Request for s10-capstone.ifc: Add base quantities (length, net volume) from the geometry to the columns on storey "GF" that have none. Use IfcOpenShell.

First a look at what the model holds.

```python
import ifcopenshell
import ifcopenshell.util.element
import ifcopenshell.util.unit

model = ifcopenshell.open("s10-capstone.ifc")
print(model.schema)
for unit_type in ("LENGTHUNIT", "AREAUNIT", "VOLUMEUNIT"):
    print(unit_type, ifcopenshell.util.unit.calculate_unit_scale(model, unit_type))
storey = next(s for s in model.by_type("IfcBuildingStorey") if s.Name == "GF")
columns = [e for e in ifcopenshell.util.element.get_decomposition(storey) if e.is_a("IfcColumn")]
for e in sorted(columns, key=lambda e: e.id()):
    print(e.id(), e.is_a(), e.Name, list(ifcopenshell.util.element.get_psets(e, qtos_only=True)), sep=" | ")
```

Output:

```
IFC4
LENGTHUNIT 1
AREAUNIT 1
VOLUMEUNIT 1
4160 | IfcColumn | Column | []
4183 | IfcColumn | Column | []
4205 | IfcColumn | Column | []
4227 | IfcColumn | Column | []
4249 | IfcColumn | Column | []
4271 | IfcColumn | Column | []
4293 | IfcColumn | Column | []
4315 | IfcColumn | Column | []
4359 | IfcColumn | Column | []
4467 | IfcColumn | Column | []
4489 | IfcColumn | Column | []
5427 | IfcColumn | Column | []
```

```python
import ifcopenshell
import ifcopenshell.api.pset
import ifcopenshell.geom
import ifcopenshell.util.element
import ifcopenshell.util.shape
import ifcopenshell.util.unit

model = ifcopenshell.open("s10-capstone.ifc")
unit_scale = ifcopenshell.util.unit.calculate_unit_scale(model)
volume_scale = ifcopenshell.util.unit.calculate_unit_scale(model, "VOLUMEUNIT")
settings = ifcopenshell.geom.settings()

storey = next(s for s in model.by_type("IfcBuildingStorey") if s.Name == "GF")
columns = [e for e in ifcopenshell.util.element.get_decomposition(storey) if e.is_a("IfcColumn")]

for e in sorted(columns, key=lambda e: e.id()):
    if ifcopenshell.util.element.get_psets(e, qtos_only=True, should_inherit=False):
        continue
    # Geometry comes back in metres, in the element's own axes.
    shape = ifcopenshell.geom.create_shape(settings, e)
    values = {
        "Length": ifcopenshell.util.shape.get_z(shape.geometry) / unit_scale,
        "NetVolume": ifcopenshell.util.shape.get_volume(shape.geometry) / volume_scale,
    }
    qto = ifcopenshell.api.pset.add_qto(model, product=e, name="Qto_ColumnBaseQuantities")
    ifcopenshell.api.pset.edit_qto(model, qto=qto, properties=values)
    print(e.id(), {k: round(v, 3) for k, v in values.items()})

model.write("s10-capstone_updated.ifc")
```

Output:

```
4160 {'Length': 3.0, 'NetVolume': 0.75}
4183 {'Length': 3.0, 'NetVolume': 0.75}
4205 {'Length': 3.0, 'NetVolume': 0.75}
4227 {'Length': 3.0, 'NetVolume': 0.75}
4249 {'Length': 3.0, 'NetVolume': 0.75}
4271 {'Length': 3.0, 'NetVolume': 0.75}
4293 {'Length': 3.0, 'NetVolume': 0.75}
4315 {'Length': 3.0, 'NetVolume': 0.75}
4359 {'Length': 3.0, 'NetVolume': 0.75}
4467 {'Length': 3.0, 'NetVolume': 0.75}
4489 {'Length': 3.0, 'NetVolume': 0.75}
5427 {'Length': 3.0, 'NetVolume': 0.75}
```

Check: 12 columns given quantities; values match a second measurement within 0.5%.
